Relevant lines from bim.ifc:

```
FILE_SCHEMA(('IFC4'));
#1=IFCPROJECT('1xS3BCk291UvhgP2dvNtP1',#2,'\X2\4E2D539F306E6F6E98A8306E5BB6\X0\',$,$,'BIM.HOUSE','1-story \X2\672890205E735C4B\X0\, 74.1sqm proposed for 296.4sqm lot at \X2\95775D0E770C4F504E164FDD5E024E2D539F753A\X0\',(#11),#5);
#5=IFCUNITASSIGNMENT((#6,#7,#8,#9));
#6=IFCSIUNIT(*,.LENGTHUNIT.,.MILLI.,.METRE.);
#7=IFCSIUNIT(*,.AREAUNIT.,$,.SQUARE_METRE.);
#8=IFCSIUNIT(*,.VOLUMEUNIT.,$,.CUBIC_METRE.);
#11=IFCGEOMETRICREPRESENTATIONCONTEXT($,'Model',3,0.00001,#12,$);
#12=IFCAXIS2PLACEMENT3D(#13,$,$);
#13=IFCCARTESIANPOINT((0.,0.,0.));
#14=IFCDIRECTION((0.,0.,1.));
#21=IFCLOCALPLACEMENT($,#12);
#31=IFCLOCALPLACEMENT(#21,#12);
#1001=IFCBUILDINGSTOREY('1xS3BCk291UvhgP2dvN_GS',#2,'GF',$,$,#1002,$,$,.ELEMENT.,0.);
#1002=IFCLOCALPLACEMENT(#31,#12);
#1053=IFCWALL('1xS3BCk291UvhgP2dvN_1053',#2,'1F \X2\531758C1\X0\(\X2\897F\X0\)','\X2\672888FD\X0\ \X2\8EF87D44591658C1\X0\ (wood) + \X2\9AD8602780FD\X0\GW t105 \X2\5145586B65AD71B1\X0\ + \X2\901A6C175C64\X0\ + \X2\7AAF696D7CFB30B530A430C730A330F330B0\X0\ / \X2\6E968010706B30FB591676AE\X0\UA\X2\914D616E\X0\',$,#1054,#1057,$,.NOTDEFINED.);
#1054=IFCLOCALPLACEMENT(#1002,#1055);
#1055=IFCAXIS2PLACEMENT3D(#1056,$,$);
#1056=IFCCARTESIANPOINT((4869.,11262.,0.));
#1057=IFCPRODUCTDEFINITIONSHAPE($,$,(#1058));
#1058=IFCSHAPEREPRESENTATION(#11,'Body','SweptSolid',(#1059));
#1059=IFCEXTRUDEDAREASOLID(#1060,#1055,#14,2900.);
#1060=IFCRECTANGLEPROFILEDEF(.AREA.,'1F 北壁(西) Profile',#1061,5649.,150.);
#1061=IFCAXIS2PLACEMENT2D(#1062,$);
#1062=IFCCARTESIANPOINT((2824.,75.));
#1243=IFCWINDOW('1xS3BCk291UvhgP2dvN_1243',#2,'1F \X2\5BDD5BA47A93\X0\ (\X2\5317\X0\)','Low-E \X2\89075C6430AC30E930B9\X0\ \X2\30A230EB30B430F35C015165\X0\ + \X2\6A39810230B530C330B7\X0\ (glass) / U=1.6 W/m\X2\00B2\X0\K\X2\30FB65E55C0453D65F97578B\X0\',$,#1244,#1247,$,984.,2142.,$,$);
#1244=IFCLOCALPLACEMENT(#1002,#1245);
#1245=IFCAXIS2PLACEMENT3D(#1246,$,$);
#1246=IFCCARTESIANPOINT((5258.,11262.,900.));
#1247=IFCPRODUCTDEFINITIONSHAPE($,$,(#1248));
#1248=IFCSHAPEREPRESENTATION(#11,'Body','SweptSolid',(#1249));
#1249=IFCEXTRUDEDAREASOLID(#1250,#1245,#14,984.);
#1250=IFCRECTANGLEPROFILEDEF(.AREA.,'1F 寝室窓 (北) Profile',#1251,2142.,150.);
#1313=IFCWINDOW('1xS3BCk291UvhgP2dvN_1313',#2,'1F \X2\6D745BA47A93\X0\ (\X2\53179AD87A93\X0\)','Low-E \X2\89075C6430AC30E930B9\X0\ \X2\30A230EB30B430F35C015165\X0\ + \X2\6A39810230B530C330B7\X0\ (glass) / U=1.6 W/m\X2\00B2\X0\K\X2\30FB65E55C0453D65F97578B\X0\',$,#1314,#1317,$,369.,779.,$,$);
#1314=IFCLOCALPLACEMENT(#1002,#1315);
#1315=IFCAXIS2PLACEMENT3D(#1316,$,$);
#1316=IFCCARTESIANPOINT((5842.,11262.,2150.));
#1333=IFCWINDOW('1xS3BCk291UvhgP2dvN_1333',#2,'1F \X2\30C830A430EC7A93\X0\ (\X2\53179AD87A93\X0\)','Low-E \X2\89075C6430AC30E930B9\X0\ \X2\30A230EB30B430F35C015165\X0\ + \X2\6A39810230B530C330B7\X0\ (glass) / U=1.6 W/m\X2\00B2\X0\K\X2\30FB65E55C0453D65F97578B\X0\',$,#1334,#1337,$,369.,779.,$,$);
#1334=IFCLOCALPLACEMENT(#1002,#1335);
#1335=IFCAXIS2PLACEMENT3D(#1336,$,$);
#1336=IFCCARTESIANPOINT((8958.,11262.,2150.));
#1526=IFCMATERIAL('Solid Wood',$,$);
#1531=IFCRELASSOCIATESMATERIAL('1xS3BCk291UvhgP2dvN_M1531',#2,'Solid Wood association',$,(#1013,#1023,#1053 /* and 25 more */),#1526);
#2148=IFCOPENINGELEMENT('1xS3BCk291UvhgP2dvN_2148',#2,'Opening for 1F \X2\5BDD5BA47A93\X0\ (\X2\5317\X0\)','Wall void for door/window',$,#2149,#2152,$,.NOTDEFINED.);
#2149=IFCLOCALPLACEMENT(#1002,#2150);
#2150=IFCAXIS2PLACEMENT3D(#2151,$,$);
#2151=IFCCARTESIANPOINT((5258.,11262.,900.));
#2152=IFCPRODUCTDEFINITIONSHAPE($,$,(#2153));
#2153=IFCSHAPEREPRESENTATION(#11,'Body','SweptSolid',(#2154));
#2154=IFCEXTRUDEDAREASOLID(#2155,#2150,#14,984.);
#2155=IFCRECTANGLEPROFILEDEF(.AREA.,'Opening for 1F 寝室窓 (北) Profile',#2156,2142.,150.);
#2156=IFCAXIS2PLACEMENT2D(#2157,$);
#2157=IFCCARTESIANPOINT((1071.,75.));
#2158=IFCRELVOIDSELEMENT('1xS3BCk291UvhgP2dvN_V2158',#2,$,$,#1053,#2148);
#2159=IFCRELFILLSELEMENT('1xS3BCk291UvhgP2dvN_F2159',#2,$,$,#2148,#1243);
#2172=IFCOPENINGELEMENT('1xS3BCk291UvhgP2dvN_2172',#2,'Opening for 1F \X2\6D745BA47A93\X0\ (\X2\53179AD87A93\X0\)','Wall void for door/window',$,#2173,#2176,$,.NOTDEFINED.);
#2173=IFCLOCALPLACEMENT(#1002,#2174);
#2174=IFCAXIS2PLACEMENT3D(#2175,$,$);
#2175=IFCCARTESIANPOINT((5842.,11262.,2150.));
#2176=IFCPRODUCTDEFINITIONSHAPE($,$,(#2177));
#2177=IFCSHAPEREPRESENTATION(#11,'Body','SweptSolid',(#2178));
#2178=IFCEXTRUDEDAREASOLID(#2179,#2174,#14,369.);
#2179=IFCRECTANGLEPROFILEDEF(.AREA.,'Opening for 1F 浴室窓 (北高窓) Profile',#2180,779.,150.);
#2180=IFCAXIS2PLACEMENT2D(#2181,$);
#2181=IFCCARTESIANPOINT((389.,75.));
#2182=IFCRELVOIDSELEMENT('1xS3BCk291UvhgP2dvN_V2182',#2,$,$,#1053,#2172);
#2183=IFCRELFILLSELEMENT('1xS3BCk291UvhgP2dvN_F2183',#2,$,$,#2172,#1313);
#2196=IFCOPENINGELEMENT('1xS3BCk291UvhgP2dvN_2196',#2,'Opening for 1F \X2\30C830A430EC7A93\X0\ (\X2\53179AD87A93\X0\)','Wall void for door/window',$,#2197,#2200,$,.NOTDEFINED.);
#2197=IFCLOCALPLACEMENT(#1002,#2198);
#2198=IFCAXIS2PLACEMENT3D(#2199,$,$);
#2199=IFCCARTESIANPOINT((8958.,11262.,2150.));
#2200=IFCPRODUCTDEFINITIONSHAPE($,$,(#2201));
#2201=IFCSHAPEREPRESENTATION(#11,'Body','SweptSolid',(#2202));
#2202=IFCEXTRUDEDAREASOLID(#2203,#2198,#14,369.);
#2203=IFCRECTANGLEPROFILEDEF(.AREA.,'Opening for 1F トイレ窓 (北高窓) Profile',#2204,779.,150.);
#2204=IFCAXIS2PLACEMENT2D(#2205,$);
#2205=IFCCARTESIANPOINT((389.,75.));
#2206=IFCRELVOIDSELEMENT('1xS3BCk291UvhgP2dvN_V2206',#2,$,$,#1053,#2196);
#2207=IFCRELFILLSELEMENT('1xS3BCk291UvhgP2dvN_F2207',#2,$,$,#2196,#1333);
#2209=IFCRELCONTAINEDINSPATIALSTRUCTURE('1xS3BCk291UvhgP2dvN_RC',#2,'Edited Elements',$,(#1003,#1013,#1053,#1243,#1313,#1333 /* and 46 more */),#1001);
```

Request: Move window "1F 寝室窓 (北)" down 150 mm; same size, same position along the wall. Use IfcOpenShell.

```python
import numpy as np
import ifcopenshell
import ifcopenshell.api.geometry
import ifcopenshell.util.placement
import ifcopenshell.util.unit

model = ifcopenshell.open("bim.ifc")
unit_scale = ifcopenshell.util.unit.calculate_unit_scale(model)

window = model.by_guid("1xS3BCk291UvhgP2dvN_1243")
opening = window.FillsVoids[0].RelatingOpeningElement
dz = -0.15 / unit_scale

shift = np.array([0.0, 0.0, dz])
# The window is not placed relative to its opening, so move both.
for product in (opening, window):
    matrix = ifcopenshell.util.placement.get_local_placement(product.ObjectPlacement)
    matrix[:3, 3] += shift
    ifcopenshell.api.geometry.edit_object_placement(model, product=product, matrix=matrix, is_si=False)

print(f"moved by {dz * unit_scale:+.3f} m")

model.write("bim_v2.ifc")
```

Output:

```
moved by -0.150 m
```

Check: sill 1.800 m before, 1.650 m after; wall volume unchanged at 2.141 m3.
